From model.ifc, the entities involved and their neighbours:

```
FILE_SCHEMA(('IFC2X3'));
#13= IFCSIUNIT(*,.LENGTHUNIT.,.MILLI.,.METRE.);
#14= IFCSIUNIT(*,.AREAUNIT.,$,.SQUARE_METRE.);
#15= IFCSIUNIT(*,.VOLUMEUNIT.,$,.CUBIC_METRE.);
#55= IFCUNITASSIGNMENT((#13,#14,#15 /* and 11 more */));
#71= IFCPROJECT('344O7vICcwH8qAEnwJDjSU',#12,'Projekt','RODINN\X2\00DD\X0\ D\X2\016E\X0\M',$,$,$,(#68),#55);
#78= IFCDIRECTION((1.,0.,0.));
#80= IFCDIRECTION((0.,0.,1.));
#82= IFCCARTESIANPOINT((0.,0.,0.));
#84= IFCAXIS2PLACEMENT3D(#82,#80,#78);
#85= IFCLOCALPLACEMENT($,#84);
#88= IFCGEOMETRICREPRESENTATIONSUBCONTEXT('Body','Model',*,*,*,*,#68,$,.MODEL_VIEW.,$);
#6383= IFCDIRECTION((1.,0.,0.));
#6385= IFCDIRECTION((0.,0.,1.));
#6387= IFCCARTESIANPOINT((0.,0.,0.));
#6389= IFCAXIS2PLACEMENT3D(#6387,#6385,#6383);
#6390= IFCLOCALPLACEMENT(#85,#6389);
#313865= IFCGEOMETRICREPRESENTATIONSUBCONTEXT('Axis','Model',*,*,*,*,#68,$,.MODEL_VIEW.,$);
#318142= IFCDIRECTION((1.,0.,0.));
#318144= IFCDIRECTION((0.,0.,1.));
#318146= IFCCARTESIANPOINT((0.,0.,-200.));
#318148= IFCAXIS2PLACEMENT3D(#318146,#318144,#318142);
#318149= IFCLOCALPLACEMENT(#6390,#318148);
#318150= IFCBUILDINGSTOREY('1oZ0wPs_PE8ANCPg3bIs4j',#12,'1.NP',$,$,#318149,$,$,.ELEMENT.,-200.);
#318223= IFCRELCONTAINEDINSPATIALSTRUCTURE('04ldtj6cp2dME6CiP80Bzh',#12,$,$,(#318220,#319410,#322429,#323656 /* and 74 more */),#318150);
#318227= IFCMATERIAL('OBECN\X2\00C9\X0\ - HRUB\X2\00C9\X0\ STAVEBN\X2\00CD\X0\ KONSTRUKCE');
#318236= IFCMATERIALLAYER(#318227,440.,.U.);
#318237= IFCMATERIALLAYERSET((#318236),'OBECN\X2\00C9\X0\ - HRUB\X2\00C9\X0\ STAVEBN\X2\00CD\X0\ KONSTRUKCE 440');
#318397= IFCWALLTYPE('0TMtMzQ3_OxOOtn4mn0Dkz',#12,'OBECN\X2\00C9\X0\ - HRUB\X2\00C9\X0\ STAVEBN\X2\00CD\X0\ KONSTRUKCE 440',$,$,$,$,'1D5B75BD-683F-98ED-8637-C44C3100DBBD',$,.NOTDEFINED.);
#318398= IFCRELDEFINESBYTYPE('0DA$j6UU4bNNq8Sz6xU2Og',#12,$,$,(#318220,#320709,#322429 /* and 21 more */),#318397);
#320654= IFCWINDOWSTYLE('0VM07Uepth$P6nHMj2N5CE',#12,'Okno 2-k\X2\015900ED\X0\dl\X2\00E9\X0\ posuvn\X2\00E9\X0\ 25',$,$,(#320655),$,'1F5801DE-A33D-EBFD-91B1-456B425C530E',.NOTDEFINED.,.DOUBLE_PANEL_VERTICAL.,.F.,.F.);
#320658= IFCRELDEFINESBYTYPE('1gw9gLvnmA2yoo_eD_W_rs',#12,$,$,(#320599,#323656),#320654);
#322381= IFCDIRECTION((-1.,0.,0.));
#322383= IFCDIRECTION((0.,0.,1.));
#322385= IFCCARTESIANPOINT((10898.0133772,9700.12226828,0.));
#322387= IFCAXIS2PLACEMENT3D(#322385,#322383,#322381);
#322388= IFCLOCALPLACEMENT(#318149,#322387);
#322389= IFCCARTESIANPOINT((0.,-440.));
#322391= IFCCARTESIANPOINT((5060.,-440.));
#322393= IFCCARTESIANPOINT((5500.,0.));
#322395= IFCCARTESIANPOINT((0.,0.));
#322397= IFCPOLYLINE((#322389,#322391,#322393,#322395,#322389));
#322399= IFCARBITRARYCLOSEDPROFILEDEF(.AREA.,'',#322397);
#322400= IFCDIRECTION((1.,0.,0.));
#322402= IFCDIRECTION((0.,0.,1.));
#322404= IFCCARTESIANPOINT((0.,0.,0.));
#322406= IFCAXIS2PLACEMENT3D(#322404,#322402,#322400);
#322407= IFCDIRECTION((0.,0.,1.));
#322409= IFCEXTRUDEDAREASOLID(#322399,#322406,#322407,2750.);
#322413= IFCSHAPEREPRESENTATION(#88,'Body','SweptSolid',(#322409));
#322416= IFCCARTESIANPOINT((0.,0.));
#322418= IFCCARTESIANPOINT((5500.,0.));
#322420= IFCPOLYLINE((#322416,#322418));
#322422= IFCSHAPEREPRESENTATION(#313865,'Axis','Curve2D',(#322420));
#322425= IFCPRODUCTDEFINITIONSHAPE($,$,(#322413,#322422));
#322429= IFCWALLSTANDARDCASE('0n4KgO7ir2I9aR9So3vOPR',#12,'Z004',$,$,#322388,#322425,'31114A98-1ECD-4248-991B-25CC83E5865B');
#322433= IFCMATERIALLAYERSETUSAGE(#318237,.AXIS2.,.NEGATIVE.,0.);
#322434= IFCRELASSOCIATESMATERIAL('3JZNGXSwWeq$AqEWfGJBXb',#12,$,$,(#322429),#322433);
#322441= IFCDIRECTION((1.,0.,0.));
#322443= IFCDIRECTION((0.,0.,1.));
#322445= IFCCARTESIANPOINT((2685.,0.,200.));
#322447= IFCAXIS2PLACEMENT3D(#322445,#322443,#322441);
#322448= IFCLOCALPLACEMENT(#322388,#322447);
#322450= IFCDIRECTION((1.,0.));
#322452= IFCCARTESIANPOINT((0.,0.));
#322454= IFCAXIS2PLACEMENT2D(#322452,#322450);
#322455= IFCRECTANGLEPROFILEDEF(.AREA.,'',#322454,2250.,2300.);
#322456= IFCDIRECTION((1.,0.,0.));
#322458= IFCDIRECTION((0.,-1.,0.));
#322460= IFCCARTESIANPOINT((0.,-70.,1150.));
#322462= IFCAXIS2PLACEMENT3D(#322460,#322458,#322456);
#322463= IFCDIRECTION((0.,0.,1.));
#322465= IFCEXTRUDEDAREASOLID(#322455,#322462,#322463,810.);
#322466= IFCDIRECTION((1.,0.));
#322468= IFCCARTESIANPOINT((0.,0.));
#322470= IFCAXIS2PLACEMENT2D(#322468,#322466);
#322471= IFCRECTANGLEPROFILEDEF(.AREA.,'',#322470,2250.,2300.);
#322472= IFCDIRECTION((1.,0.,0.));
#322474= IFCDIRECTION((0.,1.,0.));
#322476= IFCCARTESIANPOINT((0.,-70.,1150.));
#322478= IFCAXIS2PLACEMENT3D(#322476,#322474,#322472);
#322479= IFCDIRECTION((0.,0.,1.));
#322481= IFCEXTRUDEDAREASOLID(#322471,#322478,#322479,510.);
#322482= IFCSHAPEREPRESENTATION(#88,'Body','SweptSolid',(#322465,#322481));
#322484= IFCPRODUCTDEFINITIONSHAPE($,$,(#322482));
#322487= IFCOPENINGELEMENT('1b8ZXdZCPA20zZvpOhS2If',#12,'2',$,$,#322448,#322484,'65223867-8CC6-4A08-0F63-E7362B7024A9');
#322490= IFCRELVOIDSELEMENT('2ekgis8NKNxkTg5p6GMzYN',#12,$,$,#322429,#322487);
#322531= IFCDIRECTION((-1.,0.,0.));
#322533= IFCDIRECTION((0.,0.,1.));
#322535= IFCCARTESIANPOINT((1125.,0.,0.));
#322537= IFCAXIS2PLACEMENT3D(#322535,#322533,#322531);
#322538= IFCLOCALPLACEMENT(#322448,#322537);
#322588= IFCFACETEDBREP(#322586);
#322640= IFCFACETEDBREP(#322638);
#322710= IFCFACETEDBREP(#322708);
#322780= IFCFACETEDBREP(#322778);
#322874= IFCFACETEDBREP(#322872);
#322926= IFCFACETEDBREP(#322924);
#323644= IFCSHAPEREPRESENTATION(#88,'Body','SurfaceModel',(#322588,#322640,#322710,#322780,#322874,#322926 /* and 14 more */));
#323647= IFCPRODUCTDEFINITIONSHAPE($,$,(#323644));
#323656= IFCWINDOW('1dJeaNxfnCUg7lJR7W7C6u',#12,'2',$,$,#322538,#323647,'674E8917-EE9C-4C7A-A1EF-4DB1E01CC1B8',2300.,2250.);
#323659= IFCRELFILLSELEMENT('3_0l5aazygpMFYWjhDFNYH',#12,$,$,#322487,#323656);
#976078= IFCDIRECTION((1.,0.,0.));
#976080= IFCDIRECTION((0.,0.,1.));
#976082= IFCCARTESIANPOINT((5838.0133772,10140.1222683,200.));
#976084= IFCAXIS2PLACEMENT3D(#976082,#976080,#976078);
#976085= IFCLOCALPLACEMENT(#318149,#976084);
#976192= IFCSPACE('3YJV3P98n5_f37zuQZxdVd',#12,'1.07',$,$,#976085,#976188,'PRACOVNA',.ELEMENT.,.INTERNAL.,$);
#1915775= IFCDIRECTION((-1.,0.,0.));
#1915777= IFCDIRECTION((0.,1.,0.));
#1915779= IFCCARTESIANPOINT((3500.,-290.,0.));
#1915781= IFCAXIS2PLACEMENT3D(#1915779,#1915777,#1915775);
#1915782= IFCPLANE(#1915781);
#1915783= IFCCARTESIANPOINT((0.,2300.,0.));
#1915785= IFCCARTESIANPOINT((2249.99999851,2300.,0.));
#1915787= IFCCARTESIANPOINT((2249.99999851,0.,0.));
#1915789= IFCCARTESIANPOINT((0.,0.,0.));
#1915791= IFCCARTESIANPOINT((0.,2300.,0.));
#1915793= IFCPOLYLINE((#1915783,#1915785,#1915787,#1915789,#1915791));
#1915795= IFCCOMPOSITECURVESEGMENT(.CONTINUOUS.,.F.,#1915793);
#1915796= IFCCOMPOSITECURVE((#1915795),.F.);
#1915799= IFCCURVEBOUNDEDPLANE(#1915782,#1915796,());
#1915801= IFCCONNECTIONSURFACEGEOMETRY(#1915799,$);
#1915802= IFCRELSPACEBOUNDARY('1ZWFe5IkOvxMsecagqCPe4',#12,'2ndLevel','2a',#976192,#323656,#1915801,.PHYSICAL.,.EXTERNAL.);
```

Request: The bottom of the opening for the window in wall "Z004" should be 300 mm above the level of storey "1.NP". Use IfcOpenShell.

```python
import numpy as np
import ifcopenshell
import ifcopenshell.api.geometry
import ifcopenshell.geom
import ifcopenshell.util.element
import ifcopenshell.util.placement
import ifcopenshell.util.shape
import ifcopenshell.util.unit

model = ifcopenshell.open("model.ifc")
unit_scale = ifcopenshell.util.unit.calculate_unit_scale(model)

window = model.by_guid("1dJeaNxfnCUg7lJR7W7C6u")
opening = window.FillsVoids[0].RelatingOpeningElement
storey = ifcopenshell.util.element.get_container(window, ifc_class="IfcBuildingStorey")
level = ifcopenshell.util.placement.get_local_placement(storey.ObjectPlacement)[2, 3]

# The opening's origin need not be at the sill, so measure its lowest point.
shape = ifcopenshell.geom.create_shape(ifcopenshell.geom.settings(), opening)
bottom = ifcopenshell.util.shape.get_shape_bottom_elevation(shape, shape.geometry) / unit_scale
dz = level + 300.0 - bottom

shift = np.array([0.0, 0.0, dz])
# The window is placed relative to its opening, so it follows when the opening moves.
matrix = ifcopenshell.util.placement.get_local_placement(opening.ObjectPlacement)
matrix[:3, 3] += shift
ifcopenshell.api.geometry.edit_object_placement(
    model, product=opening, matrix=matrix, is_si=False, should_transform_children=True
)

# Space boundary surfaces are stored in each space's coordinates; move them too.
for rel in window.ProvidesBoundaries:
    if not rel.ConnectionGeometry:
        continue
    surface = rel.ConnectionGeometry.SurfaceOnRelatingElement.BasisSurface
    space_matrix = ifcopenshell.util.placement.get_local_placement(rel.RelatingSpace.ObjectPlacement)
    point = np.array(surface.Position.Location.Coordinates) + space_matrix[:3, :3].T @ shift
    surface.Position = model.createIfcAxis2Placement3D(
        model.createIfcCartesianPoint(point.tolist()), surface.Position.Axis, surface.Position.RefDirection
    )

print(f"moved by {dz * unit_scale:+.3f} m")

model.write("model_edited.ifc")
```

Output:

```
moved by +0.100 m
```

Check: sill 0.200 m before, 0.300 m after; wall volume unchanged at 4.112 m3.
